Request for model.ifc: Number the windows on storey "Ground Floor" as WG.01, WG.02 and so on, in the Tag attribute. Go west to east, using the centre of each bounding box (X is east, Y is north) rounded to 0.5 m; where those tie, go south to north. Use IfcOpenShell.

First a look at what the model holds.

```python
import ifcopenshell
import ifcopenshell.util.element
import ifcopenshell.util.placement

model = ifcopenshell.open("model.ifc")
print(model.schema)
storey = next(s for s in model.by_type("IfcBuildingStorey") if s.Name == "Ground Floor")
windows = [e for e in ifcopenshell.util.element.get_decomposition(storey) if e.is_a("IfcWindow")]
for e in sorted(windows, key=lambda e: e.id()):
    origin = ifcopenshell.util.placement.get_local_placement(e.ObjectPlacement)[:3, 3]
    print(e.id(), e.Tag, e.Name, origin.round(2) + 0.0, sep=" | ")
```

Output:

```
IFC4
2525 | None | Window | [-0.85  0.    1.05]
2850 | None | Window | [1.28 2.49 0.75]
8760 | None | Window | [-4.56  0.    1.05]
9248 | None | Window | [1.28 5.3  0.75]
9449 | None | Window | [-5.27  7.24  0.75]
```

```python
import ifcopenshell
import ifcopenshell.geom
import ifcopenshell.util.element
import ifcopenshell.util.shape

model = ifcopenshell.open("model.ifc")
settings = ifcopenshell.geom.settings()
settings.set("use-world-coords", True)


def centre(element):
    shape = ifcopenshell.geom.create_shape(settings, element)
    return ifcopenshell.util.shape.get_bbox_centroid(shape.geometry)


storey = next(s for s in model.by_type("IfcBuildingStorey") if s.Name == "Ground Floor")
windows = [e for e in ifcopenshell.util.element.get_decomposition(storey) if e.is_a("IfcWindow")]

# Insertion points can sit at a corner or the storey origin, so sort by the geometry (in metres).
centres = {e: centre(e) for e in windows}
windows.sort(key=lambda e: (round(centres[e][0] / 0.5), centres[e][1]))

for i, e in enumerate(windows, start=1):
    number = f"WG.{i:02d}"
    e.Tag = number
    print(e.id(), number)

model.write("model-out.ifc")
```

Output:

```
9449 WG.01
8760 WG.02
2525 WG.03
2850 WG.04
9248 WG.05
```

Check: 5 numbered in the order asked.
